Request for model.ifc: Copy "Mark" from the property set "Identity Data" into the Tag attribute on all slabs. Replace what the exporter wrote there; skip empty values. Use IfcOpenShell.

First a look at what the model holds.

```python
import ifcopenshell
import ifcopenshell.util.element

model = ifcopenshell.open("model.ifc")
print(model.schema)
slabs = model.by_type("IfcSlab")
print(len(slabs), "slabs")
for e in slabs[:8]:
    source = ifcopenshell.util.element.get_pset(e, "Identity Data", "Mark")
    target = e.Tag
    print(e.id(), repr(source), repr(target), sep=" | ")
```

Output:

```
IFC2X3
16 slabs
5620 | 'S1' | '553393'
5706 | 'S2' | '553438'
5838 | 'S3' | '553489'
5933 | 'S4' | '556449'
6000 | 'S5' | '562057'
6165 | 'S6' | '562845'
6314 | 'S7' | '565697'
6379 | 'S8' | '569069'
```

```python
import ifcopenshell
import ifcopenshell.util.element

model = ifcopenshell.open("model.ifc")

count = 0
for e in model.by_type("IfcSlab"):
    value = ifcopenshell.util.element.get_pset(e, "Identity Data", "Mark")
    current = e.Tag
    if not value or not value.strip() or current == value:
        continue
    e.Tag = value
    count += 1

print(count, "slabs updated")

model.write("model-out.ifc")
```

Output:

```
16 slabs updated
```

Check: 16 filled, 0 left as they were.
